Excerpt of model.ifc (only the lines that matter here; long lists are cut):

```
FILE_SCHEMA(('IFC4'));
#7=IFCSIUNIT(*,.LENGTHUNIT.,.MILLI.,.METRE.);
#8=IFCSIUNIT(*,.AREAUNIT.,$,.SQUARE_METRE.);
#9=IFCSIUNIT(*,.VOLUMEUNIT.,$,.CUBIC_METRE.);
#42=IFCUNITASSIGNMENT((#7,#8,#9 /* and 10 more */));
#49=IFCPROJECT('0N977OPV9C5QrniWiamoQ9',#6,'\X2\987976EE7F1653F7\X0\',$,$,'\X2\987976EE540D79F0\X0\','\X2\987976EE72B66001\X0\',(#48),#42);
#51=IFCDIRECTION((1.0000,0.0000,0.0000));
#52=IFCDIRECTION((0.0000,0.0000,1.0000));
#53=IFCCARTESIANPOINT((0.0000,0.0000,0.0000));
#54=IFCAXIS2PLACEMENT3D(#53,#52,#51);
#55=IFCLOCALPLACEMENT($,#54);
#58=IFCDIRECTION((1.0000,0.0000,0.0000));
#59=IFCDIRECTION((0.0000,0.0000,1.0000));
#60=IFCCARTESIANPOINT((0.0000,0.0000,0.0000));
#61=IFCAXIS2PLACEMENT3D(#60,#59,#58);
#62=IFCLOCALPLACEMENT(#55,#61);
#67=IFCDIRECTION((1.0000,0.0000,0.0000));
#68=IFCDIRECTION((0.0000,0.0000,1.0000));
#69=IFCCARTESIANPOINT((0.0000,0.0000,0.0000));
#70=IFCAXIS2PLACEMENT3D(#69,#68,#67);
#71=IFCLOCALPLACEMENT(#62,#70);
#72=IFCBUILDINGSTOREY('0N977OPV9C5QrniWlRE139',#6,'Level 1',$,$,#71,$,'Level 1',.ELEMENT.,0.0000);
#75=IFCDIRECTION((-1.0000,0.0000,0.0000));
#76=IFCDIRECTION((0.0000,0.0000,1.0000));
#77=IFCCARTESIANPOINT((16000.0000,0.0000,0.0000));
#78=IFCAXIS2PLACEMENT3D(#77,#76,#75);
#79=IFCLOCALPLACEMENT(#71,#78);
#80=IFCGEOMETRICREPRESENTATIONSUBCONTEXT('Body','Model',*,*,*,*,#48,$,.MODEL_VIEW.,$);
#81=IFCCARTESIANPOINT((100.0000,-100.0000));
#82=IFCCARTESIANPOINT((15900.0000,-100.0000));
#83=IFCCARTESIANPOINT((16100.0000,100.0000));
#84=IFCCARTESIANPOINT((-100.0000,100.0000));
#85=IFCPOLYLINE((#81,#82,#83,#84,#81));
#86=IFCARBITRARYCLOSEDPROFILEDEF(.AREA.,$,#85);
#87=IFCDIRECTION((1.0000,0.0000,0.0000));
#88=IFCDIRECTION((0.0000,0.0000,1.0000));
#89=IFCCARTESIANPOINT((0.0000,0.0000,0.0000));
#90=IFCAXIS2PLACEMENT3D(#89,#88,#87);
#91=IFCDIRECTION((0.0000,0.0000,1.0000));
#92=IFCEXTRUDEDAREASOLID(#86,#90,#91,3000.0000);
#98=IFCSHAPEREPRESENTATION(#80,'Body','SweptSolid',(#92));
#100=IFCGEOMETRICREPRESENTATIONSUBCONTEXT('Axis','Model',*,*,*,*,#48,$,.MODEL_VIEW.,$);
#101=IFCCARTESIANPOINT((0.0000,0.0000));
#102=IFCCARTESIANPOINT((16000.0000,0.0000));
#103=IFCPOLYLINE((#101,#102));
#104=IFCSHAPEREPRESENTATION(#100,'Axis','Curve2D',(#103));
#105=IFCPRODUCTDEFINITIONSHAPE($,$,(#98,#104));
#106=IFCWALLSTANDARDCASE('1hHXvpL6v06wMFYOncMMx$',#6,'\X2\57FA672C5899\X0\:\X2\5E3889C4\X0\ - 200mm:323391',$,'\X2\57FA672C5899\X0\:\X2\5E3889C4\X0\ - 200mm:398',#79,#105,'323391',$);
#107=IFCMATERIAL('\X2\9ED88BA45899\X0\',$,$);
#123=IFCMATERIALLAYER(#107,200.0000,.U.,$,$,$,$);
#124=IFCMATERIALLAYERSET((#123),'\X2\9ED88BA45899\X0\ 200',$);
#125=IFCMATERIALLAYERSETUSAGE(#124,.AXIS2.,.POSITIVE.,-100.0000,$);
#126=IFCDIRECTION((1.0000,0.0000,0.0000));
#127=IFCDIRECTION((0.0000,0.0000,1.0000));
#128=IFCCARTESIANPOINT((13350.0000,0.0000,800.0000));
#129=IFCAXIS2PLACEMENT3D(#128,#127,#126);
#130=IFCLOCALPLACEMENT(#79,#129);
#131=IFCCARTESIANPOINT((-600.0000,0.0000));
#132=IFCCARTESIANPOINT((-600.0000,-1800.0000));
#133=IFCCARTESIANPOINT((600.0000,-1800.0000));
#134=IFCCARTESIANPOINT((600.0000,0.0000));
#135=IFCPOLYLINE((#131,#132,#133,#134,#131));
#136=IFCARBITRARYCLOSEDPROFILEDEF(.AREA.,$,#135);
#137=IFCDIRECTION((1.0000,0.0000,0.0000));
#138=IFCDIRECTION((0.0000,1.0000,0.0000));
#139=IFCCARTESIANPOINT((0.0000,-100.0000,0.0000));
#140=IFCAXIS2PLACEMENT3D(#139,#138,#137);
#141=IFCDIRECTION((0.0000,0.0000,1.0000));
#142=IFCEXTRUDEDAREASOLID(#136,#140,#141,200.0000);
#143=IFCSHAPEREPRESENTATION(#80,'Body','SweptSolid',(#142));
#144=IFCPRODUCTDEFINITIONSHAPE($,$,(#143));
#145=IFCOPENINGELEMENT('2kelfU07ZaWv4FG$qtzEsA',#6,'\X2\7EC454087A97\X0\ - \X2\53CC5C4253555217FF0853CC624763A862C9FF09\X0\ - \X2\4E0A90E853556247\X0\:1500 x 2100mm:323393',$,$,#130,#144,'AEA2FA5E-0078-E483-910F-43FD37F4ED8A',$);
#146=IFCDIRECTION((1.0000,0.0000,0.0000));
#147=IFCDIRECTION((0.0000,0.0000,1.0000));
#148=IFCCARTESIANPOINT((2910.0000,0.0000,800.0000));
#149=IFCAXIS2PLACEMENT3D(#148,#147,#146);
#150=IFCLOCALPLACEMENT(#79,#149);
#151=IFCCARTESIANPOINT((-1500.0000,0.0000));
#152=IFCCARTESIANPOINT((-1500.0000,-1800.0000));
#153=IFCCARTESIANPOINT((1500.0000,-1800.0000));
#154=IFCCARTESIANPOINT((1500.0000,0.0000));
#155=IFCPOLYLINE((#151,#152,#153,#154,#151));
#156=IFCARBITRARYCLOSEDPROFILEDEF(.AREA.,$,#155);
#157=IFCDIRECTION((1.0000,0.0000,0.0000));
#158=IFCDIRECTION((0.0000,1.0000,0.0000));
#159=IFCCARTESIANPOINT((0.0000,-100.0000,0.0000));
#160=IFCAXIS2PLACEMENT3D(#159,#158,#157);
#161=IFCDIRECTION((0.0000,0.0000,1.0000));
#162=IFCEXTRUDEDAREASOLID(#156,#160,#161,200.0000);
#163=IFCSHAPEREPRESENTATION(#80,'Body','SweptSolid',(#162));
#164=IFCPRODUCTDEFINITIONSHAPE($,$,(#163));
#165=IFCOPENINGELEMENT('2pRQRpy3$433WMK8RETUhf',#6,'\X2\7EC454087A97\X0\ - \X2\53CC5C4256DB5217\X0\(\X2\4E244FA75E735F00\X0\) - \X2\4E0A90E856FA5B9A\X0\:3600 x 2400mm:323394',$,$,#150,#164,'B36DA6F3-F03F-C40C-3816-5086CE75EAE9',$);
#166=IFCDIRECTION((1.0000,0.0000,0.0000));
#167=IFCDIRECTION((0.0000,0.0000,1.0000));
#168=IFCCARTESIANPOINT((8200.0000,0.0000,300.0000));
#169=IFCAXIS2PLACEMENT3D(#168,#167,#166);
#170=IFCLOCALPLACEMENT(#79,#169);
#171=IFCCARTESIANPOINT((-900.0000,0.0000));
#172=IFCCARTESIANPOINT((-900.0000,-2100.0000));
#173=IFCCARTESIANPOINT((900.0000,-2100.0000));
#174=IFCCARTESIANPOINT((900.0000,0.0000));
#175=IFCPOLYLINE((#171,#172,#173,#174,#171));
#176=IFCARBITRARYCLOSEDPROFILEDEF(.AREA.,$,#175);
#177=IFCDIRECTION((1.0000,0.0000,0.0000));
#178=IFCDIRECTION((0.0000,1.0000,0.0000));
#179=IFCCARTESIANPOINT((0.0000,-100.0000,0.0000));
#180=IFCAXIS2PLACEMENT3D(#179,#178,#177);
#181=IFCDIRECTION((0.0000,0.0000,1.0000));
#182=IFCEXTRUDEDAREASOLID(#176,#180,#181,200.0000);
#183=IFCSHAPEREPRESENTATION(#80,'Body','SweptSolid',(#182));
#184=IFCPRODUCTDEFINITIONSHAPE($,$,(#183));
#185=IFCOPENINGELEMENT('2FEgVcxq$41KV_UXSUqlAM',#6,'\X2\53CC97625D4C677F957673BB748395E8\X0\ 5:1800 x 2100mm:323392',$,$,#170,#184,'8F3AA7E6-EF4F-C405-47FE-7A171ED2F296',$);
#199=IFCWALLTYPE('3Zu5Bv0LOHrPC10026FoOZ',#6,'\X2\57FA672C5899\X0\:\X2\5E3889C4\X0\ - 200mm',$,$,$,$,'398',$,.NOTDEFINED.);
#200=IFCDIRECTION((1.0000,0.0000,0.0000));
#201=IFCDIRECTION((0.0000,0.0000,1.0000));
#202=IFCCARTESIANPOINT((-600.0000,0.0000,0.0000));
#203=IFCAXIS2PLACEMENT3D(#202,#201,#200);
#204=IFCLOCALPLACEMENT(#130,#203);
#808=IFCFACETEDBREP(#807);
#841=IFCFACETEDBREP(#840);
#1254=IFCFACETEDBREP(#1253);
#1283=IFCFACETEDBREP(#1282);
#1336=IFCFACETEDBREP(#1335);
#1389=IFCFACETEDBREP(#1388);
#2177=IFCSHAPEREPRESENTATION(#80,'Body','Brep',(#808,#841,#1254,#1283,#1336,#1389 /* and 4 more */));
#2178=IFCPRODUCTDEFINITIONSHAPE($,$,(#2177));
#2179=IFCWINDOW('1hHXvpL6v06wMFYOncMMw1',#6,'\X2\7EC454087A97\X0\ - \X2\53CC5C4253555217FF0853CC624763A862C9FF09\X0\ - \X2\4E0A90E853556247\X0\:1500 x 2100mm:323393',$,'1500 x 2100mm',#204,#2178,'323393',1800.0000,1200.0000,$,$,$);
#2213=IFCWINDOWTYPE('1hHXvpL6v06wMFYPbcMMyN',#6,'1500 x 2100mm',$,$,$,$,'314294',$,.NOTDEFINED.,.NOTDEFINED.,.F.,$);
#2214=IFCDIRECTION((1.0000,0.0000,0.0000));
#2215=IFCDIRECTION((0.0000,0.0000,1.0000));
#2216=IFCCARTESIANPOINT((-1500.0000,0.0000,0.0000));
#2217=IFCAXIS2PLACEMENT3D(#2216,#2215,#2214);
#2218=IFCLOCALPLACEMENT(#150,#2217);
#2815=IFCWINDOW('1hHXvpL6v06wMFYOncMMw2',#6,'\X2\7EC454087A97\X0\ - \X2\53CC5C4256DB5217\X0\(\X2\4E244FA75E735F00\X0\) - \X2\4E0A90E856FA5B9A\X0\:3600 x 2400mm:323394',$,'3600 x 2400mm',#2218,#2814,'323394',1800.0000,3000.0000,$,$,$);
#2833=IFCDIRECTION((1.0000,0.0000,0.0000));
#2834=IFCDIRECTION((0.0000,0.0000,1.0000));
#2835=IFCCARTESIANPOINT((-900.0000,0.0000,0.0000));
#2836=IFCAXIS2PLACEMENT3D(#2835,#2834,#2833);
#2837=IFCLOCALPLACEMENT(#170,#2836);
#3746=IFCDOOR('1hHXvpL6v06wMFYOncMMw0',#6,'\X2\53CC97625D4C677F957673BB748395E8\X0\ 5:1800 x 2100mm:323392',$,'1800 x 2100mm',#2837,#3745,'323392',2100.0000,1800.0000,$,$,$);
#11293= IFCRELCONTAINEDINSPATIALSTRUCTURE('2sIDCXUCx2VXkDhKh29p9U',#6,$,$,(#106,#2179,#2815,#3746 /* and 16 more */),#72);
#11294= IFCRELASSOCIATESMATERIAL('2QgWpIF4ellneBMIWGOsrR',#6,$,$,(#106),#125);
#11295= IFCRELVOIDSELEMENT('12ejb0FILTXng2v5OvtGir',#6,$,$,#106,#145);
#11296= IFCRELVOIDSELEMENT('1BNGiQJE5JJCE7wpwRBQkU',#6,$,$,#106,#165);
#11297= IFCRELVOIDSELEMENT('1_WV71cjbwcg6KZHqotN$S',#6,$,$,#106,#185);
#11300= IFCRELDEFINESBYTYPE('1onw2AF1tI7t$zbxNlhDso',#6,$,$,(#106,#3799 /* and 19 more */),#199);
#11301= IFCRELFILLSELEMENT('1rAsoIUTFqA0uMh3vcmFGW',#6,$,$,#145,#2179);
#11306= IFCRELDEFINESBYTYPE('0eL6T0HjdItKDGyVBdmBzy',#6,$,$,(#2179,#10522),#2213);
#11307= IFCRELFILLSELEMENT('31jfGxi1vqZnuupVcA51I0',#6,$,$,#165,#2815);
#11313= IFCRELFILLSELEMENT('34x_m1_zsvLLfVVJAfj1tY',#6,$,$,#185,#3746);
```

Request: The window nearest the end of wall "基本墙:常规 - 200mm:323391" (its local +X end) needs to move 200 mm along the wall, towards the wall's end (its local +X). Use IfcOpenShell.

```python
import ifcopenshell
import ifcopenshell.api.geometry
import ifcopenshell.util.placement

model = ifcopenshell.open("model.ifc")

window = model.by_id(2179)
opening = window.FillsVoids[0].RelatingOpeningElement
wall = opening.VoidsElements[0].RelatingBuildingElement

wall_matrix = ifcopenshell.util.placement.get_local_placement(wall.ObjectPlacement)
shift = wall_matrix[:3, 0] * 200.0
before = ifcopenshell.util.placement.get_local_placement(window.ObjectPlacement)[:3, 3].copy()

# The window is placed relative to its opening, so it follows when the opening moves.
matrix = ifcopenshell.util.placement.get_local_placement(opening.ObjectPlacement)
matrix[:3, 3] += shift
ifcopenshell.api.geometry.edit_object_placement(
    model, product=opening, matrix=matrix, is_si=False, should_transform_children=True
)

after = ifcopenshell.util.placement.get_local_placement(window.ObjectPlacement)[:3, 3]
print("window moved by", (after - before).round(3) + 0.0)

model.write("model_v2.ifc")
```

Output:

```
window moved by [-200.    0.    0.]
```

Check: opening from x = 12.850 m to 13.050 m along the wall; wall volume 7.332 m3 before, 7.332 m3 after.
